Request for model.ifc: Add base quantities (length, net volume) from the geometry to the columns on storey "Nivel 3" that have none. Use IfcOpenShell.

First a look at what the model holds.

```python
import ifcopenshell
import ifcopenshell.util.element
import ifcopenshell.util.unit

model = ifcopenshell.open("model.ifc")
print(model.schema)
for unit_type in ("LENGTHUNIT", "AREAUNIT", "VOLUMEUNIT"):
    print(unit_type, ifcopenshell.util.unit.calculate_unit_scale(model, unit_type))
storey = next(s for s in model.by_type("IfcBuildingStorey") if s.Name == "Nivel 3")
columns = [e for e in ifcopenshell.util.element.get_decomposition(storey) if e.is_a("IfcColumn")]
for e in sorted(columns, key=lambda e: e.id()):
    print(e.id(), e.is_a(), e.Name, list(ifcopenshell.util.element.get_psets(e, qtos_only=True)), sep=" | ")
```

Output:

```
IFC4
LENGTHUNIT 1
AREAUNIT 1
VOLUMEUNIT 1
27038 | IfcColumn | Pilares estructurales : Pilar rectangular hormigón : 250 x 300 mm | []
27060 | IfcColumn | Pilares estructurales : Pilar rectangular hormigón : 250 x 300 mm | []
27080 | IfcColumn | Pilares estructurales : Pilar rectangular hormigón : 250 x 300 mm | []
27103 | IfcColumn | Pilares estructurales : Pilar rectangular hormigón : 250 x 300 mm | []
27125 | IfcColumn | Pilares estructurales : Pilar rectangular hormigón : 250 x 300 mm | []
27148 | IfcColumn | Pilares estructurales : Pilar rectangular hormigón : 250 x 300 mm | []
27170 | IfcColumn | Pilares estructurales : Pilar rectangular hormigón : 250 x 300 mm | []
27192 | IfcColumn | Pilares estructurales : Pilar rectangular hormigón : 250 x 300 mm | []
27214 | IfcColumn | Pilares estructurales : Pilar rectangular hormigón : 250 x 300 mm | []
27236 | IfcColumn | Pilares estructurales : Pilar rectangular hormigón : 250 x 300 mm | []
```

```python
import ifcopenshell
import ifcopenshell.api.pset
import ifcopenshell.geom
import ifcopenshell.util.element
import ifcopenshell.util.shape
import ifcopenshell.util.unit

model = ifcopenshell.open("model.ifc")
unit_scale = ifcopenshell.util.unit.calculate_unit_scale(model)
volume_scale = ifcopenshell.util.unit.calculate_unit_scale(model, "VOLUMEUNIT")
settings = ifcopenshell.geom.settings()

storey = next(s for s in model.by_type("IfcBuildingStorey") if s.Name == "Nivel 3")
columns = [e for e in ifcopenshell.util.element.get_decomposition(storey) if e.is_a("IfcColumn")]

for e in sorted(columns, key=lambda e: e.id()):
    if ifcopenshell.util.element.get_psets(e, qtos_only=True, should_inherit=False):
        continue
    # Geometry comes back in metres, in the element's own axes.
    shape = ifcopenshell.geom.create_shape(settings, e)
    values = {
        "Length": ifcopenshell.util.shape.get_z(shape.geometry) / unit_scale,
        "NetVolume": ifcopenshell.util.shape.get_volume(shape.geometry) / volume_scale,
    }
    qto = ifcopenshell.api.pset.add_qto(model, product=e, name="Qto_ColumnBaseQuantities")
    ifcopenshell.api.pset.edit_qto(model, qto=qto, properties=values)
    print(e.id(), {k: round(v, 3) for k, v in values.items()})

model.write("model-out.ifc")
```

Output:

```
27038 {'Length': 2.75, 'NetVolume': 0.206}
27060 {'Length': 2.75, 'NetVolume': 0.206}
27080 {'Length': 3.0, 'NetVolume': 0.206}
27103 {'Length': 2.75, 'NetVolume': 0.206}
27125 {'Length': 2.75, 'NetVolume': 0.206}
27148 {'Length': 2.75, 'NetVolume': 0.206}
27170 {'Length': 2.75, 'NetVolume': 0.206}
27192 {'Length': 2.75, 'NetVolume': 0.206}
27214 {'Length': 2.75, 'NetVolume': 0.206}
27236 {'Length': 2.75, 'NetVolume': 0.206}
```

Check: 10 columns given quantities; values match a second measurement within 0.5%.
